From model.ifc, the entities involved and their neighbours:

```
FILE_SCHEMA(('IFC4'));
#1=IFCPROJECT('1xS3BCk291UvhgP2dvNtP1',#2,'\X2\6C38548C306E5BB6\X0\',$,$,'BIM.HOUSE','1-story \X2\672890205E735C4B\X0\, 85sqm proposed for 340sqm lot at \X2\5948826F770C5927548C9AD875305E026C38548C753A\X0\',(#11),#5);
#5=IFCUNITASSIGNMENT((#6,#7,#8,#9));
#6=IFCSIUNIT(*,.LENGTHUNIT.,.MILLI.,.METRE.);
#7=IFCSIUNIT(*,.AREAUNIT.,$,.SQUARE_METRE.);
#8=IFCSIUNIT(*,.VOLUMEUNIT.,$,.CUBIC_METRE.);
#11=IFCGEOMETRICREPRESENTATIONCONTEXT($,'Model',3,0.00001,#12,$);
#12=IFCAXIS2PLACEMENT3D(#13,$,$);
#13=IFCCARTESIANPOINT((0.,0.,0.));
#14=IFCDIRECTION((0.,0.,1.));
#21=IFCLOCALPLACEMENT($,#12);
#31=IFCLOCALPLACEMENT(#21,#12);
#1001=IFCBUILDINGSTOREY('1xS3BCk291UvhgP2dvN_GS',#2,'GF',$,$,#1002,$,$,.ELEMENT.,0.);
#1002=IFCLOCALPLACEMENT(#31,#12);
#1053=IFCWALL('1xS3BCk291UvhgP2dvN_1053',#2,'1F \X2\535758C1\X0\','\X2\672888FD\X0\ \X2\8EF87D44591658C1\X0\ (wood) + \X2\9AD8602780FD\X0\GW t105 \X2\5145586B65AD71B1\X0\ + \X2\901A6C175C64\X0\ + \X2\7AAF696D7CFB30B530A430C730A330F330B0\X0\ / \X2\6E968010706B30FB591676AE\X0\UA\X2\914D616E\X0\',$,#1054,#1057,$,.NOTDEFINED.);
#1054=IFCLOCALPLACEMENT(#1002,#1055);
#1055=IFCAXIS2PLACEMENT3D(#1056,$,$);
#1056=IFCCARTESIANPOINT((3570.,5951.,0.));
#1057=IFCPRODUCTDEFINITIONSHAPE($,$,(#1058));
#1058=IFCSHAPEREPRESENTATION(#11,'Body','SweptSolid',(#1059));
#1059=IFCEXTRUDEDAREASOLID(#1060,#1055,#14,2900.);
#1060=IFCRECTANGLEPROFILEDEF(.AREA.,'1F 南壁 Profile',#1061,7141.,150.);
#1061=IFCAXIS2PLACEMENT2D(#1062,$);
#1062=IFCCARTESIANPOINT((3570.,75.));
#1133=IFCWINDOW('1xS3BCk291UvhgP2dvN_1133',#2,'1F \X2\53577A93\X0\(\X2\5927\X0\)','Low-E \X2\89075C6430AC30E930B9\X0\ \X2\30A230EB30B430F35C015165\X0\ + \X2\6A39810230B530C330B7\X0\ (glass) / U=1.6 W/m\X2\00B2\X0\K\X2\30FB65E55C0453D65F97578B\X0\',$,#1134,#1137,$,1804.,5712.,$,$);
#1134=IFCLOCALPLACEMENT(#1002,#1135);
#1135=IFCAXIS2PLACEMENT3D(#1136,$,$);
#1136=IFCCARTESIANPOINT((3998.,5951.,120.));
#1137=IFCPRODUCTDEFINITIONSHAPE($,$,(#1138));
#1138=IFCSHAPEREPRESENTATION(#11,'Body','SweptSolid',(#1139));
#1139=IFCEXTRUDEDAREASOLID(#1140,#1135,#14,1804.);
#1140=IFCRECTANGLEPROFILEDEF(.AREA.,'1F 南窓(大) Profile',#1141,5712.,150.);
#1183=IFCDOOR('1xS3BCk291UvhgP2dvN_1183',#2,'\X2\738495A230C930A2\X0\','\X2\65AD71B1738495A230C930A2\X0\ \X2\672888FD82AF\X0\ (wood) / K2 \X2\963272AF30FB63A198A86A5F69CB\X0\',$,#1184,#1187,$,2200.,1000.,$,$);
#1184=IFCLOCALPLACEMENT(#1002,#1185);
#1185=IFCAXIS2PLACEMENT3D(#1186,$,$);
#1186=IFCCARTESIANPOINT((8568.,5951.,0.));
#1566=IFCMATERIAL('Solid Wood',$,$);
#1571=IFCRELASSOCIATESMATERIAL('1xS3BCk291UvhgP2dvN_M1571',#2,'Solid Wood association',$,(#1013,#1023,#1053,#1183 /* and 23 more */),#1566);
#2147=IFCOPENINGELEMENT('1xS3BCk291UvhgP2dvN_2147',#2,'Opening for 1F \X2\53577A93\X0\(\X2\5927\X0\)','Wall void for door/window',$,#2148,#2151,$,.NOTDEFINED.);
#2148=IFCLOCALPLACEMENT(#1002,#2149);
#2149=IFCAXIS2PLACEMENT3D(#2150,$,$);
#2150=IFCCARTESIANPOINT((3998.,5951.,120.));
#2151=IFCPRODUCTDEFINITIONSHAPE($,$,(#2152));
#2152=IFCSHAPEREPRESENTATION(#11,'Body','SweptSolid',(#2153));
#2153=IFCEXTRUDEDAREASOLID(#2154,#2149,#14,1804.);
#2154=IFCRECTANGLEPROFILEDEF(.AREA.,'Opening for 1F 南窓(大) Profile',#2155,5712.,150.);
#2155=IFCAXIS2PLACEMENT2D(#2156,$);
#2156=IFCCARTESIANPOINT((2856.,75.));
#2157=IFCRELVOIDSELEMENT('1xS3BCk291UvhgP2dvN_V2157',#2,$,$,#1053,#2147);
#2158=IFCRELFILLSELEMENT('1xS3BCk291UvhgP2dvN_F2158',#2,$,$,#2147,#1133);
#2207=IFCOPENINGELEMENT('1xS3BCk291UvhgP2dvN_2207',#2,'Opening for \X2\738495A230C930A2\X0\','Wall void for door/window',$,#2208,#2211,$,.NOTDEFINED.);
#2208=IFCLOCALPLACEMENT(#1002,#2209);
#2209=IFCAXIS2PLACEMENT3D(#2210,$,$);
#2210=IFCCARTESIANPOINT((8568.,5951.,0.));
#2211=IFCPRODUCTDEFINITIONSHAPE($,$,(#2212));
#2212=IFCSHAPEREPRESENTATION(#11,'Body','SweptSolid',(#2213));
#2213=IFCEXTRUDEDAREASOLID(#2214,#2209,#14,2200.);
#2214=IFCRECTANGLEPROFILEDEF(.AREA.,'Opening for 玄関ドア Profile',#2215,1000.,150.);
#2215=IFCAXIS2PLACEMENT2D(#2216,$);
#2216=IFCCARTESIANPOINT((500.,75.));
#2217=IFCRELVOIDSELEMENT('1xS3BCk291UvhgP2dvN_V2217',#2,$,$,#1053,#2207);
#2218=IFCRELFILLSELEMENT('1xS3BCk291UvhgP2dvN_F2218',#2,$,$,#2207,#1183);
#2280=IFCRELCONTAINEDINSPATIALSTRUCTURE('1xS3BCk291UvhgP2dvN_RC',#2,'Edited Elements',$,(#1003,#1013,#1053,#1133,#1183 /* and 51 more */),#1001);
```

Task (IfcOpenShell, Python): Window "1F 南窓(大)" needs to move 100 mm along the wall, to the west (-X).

```python
import ifcopenshell
import ifcopenshell.api.geometry
import ifcopenshell.util.placement
import ifcopenshell.util.unit

model = ifcopenshell.open("model.ifc")
unit_scale = ifcopenshell.util.unit.calculate_unit_scale(model)

window = model.by_guid("1xS3BCk291UvhgP2dvN_1133")
opening = window.FillsVoids[0].RelatingOpeningElement
wall = opening.VoidsElements[0].RelatingBuildingElement

wall_matrix = ifcopenshell.util.placement.get_local_placement(wall.ObjectPlacement)
shift = wall_matrix[:3, 0] * -0.1 / unit_scale
before = ifcopenshell.util.placement.get_local_placement(window.ObjectPlacement)[:3, 3].copy()

# The window is not placed relative to its opening, so move both.
for product in (opening, window):
    matrix = ifcopenshell.util.placement.get_local_placement(product.ObjectPlacement)
    matrix[:3, 3] += shift
    ifcopenshell.api.geometry.edit_object_placement(model, product=product, matrix=matrix, is_si=False)

after = ifcopenshell.util.placement.get_local_placement(window.ObjectPlacement)[:3, 3]
print("window moved by", (after - before).round(3) + 0.0)

model.write("model_updated.ifc")
```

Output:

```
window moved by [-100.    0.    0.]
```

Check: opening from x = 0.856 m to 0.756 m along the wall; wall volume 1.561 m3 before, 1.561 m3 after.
